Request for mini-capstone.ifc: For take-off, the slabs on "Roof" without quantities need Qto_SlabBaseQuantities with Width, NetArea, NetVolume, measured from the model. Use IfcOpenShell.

First a look at what the model holds.

```python
import ifcopenshell
import ifcopenshell.util.element
import ifcopenshell.util.unit

model = ifcopenshell.open("mini-capstone.ifc")
print(model.schema)
for unit_type in ("LENGTHUNIT", "AREAUNIT", "VOLUMEUNIT"):
    print(unit_type, ifcopenshell.util.unit.calculate_unit_scale(model, unit_type))
storey = next(s for s in model.by_type("IfcBuildingStorey") if s.Name == "Roof")
slabs = [e for e in ifcopenshell.util.element.get_decomposition(storey) if e.is_a("IfcSlab")]
for e in sorted(slabs, key=lambda e: e.id()):
    print(e.id(), e.is_a(), e.Name, list(ifcopenshell.util.element.get_psets(e, qtos_only=True)), sep=" | ")
```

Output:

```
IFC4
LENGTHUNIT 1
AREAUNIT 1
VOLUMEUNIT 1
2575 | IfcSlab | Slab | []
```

```python
import ifcopenshell
import ifcopenshell.api.pset
import ifcopenshell.geom
import ifcopenshell.util.element
import ifcopenshell.util.shape
import ifcopenshell.util.unit

model = ifcopenshell.open("mini-capstone.ifc")
unit_scale = ifcopenshell.util.unit.calculate_unit_scale(model)
area_scale = ifcopenshell.util.unit.calculate_unit_scale(model, "AREAUNIT")
volume_scale = ifcopenshell.util.unit.calculate_unit_scale(model, "VOLUMEUNIT")
settings = ifcopenshell.geom.settings()

storey = next(s for s in model.by_type("IfcBuildingStorey") if s.Name == "Roof")
slabs = [e for e in ifcopenshell.util.element.get_decomposition(storey) if e.is_a("IfcSlab")]

for e in sorted(slabs, key=lambda e: e.id()):
    if ifcopenshell.util.element.get_psets(e, qtos_only=True, should_inherit=False):
        continue
    # Geometry comes back in metres, in the element's own axes.
    shape = ifcopenshell.geom.create_shape(settings, e)
    values = {
        "Width": ifcopenshell.util.shape.get_z(shape.geometry) / unit_scale,
        "NetArea": ifcopenshell.util.shape.get_footprint_area(shape.geometry) / area_scale,
        "NetVolume": ifcopenshell.util.shape.get_volume(shape.geometry) / volume_scale,
    }
    qto = ifcopenshell.api.pset.add_qto(model, product=e, name="Qto_SlabBaseQuantities")
    ifcopenshell.api.pset.edit_qto(model, qto=qto, properties=values)
    print(e.id(), {k: round(v, 3) for k, v in values.items()})

model.write("mini-capstone_rev.ifc")
```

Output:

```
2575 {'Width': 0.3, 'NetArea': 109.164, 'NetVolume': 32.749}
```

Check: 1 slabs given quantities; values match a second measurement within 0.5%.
